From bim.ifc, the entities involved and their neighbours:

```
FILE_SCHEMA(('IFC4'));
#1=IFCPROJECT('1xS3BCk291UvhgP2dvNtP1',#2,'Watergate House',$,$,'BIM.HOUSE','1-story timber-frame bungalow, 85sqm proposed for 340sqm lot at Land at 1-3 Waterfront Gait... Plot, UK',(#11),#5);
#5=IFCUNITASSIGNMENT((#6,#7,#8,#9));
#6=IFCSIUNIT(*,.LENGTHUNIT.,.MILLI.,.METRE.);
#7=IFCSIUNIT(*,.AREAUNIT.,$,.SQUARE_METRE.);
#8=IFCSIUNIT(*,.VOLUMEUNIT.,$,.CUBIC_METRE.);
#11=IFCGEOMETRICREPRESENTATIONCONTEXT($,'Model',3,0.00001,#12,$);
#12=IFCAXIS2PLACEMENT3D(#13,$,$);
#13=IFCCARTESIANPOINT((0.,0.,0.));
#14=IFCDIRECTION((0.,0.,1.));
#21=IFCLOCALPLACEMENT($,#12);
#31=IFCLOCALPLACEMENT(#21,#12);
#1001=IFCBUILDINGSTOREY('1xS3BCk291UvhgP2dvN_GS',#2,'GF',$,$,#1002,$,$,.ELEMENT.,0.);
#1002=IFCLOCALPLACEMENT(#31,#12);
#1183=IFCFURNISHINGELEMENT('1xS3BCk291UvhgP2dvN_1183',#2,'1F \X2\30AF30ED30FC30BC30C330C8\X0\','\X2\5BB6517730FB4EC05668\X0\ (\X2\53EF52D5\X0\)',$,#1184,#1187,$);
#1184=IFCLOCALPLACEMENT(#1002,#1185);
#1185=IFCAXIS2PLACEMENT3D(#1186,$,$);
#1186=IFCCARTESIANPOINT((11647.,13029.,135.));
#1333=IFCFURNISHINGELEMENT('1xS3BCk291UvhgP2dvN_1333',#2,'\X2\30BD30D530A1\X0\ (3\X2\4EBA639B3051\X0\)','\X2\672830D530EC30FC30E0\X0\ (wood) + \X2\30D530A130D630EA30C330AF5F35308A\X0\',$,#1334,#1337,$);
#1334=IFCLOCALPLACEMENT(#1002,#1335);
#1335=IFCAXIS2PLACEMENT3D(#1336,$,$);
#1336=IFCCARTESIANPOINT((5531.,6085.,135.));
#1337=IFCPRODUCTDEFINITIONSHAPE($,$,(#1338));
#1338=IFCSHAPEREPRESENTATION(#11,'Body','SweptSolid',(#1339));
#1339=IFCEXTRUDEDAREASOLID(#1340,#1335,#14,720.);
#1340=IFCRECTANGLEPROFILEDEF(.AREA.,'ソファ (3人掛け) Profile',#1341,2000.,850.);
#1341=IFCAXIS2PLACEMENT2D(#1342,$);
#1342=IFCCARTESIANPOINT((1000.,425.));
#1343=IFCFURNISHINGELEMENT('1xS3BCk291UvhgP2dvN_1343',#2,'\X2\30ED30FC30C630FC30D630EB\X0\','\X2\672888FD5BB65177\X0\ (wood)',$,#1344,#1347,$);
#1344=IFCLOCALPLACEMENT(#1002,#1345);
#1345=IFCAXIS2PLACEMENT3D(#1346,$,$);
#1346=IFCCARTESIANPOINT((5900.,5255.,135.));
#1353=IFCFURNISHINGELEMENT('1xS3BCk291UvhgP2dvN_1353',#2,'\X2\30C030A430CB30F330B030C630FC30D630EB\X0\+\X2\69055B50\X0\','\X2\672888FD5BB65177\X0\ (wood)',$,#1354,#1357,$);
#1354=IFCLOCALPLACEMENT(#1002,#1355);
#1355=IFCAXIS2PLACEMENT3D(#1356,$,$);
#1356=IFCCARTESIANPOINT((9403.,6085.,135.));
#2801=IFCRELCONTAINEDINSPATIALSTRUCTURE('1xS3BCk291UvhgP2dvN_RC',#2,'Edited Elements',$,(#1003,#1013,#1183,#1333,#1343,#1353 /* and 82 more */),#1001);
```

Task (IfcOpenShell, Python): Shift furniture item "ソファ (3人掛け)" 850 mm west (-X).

```python
import ifcopenshell
import ifcopenshell.api.geometry
import ifcopenshell.util.placement
import ifcopenshell.util.unit

model = ifcopenshell.open("bim.ifc")
unit_scale = ifcopenshell.util.unit.calculate_unit_scale(model)

item = model.by_id(1333)
matrix = ifcopenshell.util.placement.get_local_placement(item.ObjectPlacement)
matrix[0, 3] -= 0.85 / unit_scale
ifcopenshell.api.geometry.edit_object_placement(model, product=item, matrix=matrix, is_si=False)

print(ifcopenshell.util.placement.get_local_placement(item.ObjectPlacement).round(3) + 0.0)

model.write("bim_updated.ifc")
```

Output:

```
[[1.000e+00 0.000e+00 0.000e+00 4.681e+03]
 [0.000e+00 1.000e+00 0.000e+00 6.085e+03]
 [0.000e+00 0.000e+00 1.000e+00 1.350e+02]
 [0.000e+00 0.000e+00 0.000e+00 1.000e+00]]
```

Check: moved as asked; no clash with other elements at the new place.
